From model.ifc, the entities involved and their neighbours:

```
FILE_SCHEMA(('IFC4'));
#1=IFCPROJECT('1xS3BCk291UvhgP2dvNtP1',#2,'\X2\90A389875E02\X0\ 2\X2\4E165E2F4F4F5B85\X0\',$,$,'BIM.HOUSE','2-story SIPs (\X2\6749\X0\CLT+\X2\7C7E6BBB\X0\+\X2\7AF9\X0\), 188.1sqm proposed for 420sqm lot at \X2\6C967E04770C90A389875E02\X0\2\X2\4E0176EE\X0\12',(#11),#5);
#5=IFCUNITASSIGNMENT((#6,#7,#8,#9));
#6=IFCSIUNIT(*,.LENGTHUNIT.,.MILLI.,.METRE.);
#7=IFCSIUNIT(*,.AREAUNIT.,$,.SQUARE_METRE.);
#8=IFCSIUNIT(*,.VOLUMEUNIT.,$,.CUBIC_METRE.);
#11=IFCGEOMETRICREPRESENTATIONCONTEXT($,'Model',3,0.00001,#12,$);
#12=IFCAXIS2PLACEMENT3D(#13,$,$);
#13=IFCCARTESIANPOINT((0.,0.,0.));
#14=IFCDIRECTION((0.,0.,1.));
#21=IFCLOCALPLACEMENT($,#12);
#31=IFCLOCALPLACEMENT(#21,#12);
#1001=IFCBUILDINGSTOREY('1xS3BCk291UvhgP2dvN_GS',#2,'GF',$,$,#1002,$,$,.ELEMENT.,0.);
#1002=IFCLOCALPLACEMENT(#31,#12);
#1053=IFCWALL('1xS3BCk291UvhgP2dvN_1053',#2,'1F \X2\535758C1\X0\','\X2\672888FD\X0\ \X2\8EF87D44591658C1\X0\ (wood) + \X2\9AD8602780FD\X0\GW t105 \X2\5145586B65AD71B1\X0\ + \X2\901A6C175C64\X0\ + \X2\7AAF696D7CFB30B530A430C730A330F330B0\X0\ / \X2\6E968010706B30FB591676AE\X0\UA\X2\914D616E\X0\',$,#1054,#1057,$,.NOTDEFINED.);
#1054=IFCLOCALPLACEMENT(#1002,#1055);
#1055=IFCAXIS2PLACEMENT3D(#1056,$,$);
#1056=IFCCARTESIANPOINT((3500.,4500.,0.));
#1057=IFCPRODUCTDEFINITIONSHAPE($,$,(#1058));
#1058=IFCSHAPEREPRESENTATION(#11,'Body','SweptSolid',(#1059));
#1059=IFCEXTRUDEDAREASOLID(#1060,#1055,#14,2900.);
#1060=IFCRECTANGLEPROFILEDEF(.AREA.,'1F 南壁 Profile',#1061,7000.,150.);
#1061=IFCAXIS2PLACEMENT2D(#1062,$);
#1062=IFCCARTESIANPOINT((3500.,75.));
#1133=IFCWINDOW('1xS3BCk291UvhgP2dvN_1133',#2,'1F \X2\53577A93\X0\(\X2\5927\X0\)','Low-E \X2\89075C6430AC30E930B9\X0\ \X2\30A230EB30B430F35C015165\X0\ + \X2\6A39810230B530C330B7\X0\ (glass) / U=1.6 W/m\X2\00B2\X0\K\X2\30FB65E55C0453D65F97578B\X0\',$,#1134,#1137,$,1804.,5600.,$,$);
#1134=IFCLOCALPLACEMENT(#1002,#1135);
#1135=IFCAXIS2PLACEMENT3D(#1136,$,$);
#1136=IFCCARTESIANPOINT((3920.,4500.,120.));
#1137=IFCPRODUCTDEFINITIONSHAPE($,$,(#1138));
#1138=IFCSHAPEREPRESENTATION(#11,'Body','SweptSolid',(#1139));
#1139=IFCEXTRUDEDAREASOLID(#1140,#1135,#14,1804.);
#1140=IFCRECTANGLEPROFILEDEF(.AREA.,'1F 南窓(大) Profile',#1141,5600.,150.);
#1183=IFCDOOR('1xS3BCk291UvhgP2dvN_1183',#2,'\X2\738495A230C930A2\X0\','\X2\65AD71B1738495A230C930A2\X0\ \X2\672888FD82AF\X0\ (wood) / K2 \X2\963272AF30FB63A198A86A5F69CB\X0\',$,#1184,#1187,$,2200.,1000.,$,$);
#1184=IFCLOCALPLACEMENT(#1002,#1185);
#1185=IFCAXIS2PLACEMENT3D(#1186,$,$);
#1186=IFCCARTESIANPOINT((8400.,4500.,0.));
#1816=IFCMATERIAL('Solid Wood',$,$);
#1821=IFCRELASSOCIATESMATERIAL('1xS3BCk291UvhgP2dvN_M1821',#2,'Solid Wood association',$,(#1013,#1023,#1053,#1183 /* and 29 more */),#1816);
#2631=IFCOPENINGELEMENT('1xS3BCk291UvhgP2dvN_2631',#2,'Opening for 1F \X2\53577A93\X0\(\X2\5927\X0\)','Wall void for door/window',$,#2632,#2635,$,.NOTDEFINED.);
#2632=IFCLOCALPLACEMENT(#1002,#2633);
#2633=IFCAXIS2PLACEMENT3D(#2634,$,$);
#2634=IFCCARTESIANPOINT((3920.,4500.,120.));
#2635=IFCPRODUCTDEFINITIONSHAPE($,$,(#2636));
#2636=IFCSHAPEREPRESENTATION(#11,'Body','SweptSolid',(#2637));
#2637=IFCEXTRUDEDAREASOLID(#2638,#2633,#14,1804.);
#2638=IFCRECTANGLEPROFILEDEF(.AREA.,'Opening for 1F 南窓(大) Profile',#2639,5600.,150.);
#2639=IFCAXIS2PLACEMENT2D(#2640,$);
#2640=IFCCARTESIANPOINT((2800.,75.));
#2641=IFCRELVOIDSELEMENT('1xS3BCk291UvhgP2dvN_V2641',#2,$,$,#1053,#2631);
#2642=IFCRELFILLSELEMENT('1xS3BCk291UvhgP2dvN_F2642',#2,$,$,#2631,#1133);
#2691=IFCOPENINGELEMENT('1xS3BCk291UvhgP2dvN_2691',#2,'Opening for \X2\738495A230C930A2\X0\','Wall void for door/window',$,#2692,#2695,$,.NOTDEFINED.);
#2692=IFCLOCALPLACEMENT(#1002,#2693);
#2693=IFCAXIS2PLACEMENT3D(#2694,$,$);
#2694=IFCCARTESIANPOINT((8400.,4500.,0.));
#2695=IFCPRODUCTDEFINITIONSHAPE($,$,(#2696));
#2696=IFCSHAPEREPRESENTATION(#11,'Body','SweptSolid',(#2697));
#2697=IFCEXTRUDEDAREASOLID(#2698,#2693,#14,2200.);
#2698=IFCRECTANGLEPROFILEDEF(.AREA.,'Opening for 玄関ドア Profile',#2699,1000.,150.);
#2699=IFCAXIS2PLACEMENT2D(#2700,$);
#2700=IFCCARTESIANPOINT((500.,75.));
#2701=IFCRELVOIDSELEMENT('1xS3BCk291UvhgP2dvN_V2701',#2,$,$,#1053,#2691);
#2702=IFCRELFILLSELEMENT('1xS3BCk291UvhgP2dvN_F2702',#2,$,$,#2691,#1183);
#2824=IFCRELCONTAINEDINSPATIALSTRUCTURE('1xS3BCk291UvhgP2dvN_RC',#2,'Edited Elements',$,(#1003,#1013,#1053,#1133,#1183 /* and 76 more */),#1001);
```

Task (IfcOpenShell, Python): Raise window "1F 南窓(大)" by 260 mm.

```python
import numpy as np
import ifcopenshell
import ifcopenshell.api.geometry
import ifcopenshell.util.placement
import ifcopenshell.util.unit

model = ifcopenshell.open("model.ifc")
unit_scale = ifcopenshell.util.unit.calculate_unit_scale(model)

window = model.by_id(1133)
opening = window.FillsVoids[0].RelatingOpeningElement
dz = 0.26 / unit_scale

shift = np.array([0.0, 0.0, dz])
# The window is not placed relative to its opening, so move both.
for product in (opening, window):
    matrix = ifcopenshell.util.placement.get_local_placement(product.ObjectPlacement)
    matrix[:3, 3] += shift
    ifcopenshell.api.geometry.edit_object_placement(model, product=product, matrix=matrix, is_si=False)

print(f"moved by {dz * unit_scale:+.3f} m")

model.write("model_updated.ifc")
```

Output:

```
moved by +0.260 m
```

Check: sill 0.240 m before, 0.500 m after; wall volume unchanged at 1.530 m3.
